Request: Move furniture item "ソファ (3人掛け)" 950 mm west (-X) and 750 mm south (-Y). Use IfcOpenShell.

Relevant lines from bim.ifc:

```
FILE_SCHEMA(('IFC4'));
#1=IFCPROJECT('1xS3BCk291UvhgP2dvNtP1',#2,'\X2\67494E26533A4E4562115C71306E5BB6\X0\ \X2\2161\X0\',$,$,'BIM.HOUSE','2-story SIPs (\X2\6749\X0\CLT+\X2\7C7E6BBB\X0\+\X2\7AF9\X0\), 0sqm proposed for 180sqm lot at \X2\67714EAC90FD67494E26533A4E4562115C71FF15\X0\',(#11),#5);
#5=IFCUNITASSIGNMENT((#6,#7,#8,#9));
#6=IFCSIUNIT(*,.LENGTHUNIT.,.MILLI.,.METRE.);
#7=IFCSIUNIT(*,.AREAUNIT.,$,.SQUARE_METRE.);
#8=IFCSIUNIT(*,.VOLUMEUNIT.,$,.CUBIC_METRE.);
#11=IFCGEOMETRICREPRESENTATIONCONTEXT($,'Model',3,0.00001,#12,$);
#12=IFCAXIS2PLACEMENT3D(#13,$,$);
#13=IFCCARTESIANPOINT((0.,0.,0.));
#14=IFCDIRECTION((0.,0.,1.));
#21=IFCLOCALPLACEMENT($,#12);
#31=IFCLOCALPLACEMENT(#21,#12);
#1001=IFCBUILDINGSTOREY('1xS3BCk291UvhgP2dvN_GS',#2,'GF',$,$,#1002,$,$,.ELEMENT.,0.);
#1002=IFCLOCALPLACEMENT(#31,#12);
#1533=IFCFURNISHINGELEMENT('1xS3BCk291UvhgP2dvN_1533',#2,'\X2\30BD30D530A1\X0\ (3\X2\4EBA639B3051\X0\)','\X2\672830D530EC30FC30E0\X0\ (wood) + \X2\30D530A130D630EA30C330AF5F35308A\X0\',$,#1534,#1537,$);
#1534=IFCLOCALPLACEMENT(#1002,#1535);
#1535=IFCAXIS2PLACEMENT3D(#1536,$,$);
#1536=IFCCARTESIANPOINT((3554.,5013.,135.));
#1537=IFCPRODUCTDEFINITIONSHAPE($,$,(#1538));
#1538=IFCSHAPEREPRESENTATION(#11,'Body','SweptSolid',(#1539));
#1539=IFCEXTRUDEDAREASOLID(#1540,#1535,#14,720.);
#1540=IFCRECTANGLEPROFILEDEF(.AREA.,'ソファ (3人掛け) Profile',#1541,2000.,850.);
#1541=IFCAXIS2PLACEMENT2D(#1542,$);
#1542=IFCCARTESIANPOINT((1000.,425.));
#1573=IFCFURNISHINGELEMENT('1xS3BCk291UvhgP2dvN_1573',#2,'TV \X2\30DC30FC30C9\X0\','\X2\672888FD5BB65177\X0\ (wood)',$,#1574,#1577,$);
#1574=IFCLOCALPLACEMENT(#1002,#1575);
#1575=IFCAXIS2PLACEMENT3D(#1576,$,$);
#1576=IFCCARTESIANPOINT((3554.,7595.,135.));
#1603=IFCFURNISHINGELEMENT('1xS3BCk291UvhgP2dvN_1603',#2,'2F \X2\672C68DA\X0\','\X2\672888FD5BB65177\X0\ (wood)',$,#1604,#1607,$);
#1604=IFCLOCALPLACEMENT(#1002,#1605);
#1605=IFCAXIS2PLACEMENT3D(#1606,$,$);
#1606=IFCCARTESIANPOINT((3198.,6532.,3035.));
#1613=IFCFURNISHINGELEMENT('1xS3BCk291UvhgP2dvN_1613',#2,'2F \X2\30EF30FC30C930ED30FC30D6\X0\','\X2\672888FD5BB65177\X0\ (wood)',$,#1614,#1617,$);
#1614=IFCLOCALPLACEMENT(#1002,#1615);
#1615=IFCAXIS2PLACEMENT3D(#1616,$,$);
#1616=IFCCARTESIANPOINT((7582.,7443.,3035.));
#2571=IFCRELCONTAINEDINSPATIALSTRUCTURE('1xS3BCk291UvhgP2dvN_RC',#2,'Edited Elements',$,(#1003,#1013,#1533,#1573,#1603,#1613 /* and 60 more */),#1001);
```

```python
import ifcopenshell
import ifcopenshell.api.geometry
import ifcopenshell.util.placement

model = ifcopenshell.open("bim.ifc")

item = model.by_guid("1xS3BCk291UvhgP2dvN_1533")
matrix = ifcopenshell.util.placement.get_local_placement(item.ObjectPlacement)
matrix[0, 3] -= 950.0
matrix[1, 3] -= 750.0
ifcopenshell.api.geometry.edit_object_placement(model, product=item, matrix=matrix, is_si=False)

print(ifcopenshell.util.placement.get_local_placement(item.ObjectPlacement).round(3) + 0.0)

model.write("bim_rev.ifc")
```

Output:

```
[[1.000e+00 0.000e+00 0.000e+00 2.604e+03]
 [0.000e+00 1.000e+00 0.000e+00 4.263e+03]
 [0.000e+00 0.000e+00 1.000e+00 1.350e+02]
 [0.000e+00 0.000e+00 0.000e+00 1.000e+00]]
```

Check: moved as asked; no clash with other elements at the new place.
